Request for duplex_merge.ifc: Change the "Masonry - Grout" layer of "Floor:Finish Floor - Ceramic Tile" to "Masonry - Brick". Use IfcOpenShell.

First a look at what the model holds.

```python
import ifcopenshell
import ifcopenshell.util.element

model = ifcopenshell.open("duplex_merge.ifc")
print(model.schema)
for layer_set in model.by_type("IfcMaterialLayerSet"):
    if layer_set.LayerSetName == "Floor:Finish Floor - Ceramic Tile":
        for layer in layer_set.MaterialLayers:
            print(layer.id(), layer.Material and layer.Material.Name, layer.LayerThickness, sep=" | ")
        print(len(ifcopenshell.util.element.get_elements_by_material(model, layer_set)), "elements and types use it")
print(sorted(m.Name for m in model.by_type("IfcMaterial") if m.Name)[:60])
```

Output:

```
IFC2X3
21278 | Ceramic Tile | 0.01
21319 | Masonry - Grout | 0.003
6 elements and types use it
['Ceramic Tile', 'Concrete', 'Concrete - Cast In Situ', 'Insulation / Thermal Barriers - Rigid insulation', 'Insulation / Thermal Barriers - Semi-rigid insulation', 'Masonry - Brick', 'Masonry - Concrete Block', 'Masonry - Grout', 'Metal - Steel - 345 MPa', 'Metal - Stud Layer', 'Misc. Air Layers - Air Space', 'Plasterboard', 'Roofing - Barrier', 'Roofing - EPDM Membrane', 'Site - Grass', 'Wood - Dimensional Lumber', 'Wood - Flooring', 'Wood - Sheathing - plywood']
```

```python
import ifcopenshell
import ifcopenshell.api.material

model = ifcopenshell.open("duplex_merge.ifc")

layer_set = next(s for s in model.by_type("IfcMaterialLayerSet") if s.LayerSetName == "Floor:Finish Floor - Ceramic Tile")
layer = next(l for l in layer_set.MaterialLayers if l.Material and l.Material.Name == "Masonry - Grout")
material = next(m for m in model.by_type("IfcMaterial") if m.Name == "Masonry - Brick")

# Point this one layer at the other material; renaming the old one would change it everywhere.
ifcopenshell.api.material.edit_layer(model, layer=layer, attributes={}, material=material)

print([l.Material.Name if l.Material else None for l in layer_set.MaterialLayers])

model.write("duplex_merge_edited.ifc")
```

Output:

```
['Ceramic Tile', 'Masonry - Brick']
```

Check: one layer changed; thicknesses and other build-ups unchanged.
